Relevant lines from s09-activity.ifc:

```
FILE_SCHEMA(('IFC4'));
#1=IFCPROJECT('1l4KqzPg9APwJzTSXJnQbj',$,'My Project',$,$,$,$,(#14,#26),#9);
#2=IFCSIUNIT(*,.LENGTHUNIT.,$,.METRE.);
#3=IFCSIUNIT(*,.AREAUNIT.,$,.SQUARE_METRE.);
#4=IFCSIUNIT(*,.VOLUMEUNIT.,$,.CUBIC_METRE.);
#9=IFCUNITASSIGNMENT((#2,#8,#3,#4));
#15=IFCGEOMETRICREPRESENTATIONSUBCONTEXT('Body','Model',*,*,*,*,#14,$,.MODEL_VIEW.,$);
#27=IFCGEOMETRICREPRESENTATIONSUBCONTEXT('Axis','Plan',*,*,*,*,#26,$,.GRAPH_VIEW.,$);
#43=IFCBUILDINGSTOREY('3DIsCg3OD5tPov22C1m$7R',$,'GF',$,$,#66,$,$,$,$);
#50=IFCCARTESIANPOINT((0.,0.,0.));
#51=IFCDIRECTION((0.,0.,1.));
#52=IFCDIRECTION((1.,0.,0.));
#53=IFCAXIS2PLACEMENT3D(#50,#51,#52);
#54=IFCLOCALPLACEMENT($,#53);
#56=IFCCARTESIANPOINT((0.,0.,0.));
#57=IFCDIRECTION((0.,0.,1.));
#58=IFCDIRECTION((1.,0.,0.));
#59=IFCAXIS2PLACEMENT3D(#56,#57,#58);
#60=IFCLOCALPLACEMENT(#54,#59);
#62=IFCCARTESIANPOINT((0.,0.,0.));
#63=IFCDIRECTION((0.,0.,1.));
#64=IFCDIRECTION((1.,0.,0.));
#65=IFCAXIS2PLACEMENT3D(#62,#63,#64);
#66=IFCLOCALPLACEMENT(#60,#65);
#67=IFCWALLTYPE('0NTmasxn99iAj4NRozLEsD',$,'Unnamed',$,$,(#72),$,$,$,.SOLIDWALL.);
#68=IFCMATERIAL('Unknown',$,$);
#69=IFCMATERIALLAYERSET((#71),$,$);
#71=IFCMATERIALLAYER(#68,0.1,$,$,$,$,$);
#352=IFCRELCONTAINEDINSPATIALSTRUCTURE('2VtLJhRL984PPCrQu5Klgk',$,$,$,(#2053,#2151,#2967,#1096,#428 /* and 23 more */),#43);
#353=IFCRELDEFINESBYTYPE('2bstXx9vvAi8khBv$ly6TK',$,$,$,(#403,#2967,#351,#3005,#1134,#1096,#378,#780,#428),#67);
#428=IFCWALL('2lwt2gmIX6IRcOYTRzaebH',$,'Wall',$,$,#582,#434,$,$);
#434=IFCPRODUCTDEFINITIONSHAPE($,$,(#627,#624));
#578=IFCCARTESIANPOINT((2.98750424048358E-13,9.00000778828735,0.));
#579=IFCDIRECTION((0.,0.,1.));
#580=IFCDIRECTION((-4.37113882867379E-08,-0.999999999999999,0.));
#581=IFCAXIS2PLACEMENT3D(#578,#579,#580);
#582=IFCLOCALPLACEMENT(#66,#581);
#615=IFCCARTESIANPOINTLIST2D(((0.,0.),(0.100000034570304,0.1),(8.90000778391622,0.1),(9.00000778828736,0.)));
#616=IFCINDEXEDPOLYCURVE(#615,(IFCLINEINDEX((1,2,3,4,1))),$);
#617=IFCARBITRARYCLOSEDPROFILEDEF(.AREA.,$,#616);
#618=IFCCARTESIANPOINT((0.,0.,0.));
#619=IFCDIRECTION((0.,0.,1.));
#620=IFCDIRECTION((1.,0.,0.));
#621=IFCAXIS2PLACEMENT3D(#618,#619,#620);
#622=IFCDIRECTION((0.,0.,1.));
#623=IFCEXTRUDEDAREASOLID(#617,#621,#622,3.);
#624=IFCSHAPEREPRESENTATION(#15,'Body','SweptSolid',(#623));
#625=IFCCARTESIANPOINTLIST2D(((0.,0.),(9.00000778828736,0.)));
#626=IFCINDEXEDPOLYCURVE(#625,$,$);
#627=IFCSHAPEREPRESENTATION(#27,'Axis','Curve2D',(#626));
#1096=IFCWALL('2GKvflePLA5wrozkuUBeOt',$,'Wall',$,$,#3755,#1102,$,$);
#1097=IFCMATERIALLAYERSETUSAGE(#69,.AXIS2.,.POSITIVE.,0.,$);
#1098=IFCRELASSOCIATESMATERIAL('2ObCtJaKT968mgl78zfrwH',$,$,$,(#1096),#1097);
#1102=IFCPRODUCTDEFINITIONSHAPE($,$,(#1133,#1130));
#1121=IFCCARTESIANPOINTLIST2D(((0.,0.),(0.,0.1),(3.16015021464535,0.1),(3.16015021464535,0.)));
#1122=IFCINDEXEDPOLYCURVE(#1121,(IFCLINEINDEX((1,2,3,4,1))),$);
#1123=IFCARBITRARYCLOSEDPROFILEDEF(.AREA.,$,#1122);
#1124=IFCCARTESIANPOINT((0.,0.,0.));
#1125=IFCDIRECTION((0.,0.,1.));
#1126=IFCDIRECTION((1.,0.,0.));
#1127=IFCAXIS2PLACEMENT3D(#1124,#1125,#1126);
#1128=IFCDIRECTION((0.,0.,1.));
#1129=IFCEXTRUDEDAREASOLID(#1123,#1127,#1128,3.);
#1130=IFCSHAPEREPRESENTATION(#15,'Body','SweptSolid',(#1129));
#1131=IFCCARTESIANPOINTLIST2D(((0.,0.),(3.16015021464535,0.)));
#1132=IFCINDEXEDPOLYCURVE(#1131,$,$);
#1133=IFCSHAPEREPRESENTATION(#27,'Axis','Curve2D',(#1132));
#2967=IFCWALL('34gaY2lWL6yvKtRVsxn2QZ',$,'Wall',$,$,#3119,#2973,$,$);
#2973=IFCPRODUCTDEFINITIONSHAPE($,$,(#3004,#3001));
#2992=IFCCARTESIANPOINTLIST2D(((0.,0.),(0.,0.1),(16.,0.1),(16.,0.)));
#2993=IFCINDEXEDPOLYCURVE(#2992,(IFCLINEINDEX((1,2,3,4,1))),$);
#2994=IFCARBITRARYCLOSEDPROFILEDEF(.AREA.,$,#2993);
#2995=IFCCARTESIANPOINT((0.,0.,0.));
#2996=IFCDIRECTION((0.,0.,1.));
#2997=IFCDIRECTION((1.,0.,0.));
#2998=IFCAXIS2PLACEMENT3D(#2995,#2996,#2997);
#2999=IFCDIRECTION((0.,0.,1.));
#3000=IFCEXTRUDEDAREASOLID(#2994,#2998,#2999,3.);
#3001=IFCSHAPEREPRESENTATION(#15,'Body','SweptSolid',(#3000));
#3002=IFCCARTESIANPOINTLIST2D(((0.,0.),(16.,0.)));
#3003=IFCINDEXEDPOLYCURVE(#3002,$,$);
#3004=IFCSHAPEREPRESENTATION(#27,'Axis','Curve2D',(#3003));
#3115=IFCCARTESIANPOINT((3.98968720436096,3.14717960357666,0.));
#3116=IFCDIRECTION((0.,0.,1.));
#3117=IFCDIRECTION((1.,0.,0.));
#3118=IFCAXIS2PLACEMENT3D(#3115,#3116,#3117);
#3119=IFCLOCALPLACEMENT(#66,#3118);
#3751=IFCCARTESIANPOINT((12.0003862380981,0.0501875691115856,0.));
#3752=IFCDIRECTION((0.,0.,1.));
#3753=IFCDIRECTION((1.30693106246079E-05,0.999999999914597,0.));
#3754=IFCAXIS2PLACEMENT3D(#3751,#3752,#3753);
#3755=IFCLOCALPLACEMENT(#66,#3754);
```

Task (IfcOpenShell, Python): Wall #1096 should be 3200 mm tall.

```python
import ifcopenshell
import ifcopenshell.geom
import ifcopenshell.util.representation
import ifcopenshell.util.shape
import ifcopenshell.util.unit

model = ifcopenshell.open("s09-activity.ifc")
unit_scale = ifcopenshell.util.unit.calculate_unit_scale(model)
settings = ifcopenshell.geom.settings()


def volume(element):
    """Net volume in cubic metres, openings subtracted."""
    shape = ifcopenshell.geom.create_shape(settings, element)
    return ifcopenshell.util.shape.get_volume(shape.geometry)


wall = model.by_guid("2GKvflePLA5wrozkuUBeOt")
before = volume(wall)

body = ifcopenshell.util.representation.get_representation(wall, "Model", "Body")
solid = body.Items[0]
old_height = solid.Depth
solid.Depth = 3.2 / unit_scale
after = volume(wall)

print(f"height {old_height:g} -> {solid.Depth:g}, volume {before:.3f} -> {after:.3f} m3")

model.write("s09-activity_edited.ifc")
```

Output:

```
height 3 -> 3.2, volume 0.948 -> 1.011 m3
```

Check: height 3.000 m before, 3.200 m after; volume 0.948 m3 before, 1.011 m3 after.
